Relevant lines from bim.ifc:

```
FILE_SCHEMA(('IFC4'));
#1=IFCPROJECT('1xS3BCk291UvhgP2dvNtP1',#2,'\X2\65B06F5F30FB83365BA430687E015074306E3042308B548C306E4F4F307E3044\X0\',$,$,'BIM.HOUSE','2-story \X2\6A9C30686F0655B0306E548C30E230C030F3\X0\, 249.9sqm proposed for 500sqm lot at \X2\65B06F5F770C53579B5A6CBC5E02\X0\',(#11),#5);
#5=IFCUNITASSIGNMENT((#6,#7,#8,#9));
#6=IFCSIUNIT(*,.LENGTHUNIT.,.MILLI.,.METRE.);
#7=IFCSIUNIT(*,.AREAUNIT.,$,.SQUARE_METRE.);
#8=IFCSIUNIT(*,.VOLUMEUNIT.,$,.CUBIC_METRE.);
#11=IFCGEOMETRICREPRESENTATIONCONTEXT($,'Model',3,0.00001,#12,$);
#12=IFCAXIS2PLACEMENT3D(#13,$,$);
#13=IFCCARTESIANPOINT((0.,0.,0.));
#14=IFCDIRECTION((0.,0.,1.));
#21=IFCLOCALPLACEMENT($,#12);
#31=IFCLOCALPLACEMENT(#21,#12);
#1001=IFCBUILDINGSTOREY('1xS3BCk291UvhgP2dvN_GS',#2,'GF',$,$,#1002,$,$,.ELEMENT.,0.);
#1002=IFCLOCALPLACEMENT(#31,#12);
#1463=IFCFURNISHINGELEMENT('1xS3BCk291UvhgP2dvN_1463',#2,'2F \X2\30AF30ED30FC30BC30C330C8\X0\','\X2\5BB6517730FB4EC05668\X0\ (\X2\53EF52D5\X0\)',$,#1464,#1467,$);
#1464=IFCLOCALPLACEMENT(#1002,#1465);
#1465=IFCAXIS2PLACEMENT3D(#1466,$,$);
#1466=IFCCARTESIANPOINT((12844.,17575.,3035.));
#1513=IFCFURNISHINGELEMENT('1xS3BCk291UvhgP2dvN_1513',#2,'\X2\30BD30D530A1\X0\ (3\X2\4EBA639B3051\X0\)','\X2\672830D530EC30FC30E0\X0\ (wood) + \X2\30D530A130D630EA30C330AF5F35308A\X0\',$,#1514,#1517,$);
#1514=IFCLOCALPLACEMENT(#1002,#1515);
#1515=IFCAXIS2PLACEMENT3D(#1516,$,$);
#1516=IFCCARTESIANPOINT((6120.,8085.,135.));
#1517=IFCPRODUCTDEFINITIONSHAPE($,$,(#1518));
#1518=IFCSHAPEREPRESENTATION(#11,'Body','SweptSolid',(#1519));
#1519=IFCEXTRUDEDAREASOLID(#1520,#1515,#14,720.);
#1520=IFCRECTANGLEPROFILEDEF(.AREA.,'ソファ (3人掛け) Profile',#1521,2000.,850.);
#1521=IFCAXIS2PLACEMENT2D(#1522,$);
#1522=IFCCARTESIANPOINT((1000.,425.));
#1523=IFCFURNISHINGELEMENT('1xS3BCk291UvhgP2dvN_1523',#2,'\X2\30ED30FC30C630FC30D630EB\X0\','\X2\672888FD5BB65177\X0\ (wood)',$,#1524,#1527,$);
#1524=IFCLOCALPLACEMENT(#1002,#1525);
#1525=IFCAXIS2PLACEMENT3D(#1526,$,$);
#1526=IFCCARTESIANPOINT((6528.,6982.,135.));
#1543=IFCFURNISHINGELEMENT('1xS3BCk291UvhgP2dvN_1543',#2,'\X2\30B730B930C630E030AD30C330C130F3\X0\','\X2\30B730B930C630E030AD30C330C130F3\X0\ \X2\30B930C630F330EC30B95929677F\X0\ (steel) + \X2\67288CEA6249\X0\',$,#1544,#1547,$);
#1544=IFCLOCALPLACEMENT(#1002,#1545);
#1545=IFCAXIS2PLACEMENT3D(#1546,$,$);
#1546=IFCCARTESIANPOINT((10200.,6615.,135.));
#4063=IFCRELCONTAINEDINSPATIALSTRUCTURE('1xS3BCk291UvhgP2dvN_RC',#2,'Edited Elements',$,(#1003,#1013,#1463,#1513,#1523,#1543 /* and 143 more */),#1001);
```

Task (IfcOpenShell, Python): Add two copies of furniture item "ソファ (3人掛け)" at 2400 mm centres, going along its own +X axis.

```python
import ifcopenshell
import ifcopenshell.api.geometry
import ifcopenshell.api.root
import ifcopenshell.util.element
import ifcopenshell.util.placement
import ifcopenshell.util.unit

model = ifcopenshell.open("bim.ifc")
unit_scale = ifcopenshell.util.unit.calculate_unit_scale(model)


def reuse_history(source, copy):
    """copy_class also copies each property set's owner history, people and application; keep the originals."""
    for rel in copy.IsDefinedBy:
        if rel.is_a("IfcRelDefinesByProperties") and (history := rel.RelatingPropertyDefinition.OwnerHistory):
            rel.RelatingPropertyDefinition.OwnerHistory = source.OwnerHistory
            ifcopenshell.util.element.remove_deep2(model, history)


source = model.by_id(1513)
base = ifcopenshell.util.placement.get_local_placement(source.ObjectPlacement)
step = base[:3, 0] * 2.4 / unit_scale

for i in range(1, 3):
    copy = ifcopenshell.api.root.copy_class(model, product=source)
    copy.Representation = ifcopenshell.util.element.copy_deep(
        model, source.Representation, exclude=["IfcGeometricRepresentationContext", "IfcRepresentationMap"]
    )
    reuse_history(source, copy)
    matrix = base.copy()
    matrix[:3, 3] += i * step
    print("added at", matrix[:3, 3].round(3) + 0.0)
    ifcopenshell.api.geometry.edit_object_placement(model, product=copy, matrix=matrix, is_si=False)

model.write("bim_v2.ifc")
```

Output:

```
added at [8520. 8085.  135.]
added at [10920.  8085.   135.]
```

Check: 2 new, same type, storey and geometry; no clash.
